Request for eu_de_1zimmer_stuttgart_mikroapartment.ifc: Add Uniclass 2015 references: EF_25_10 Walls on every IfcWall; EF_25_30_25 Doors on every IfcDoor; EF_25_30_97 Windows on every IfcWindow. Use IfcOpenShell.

First a look at what the model holds.

```python
import ifcopenshell

model = ifcopenshell.open("eu_de_1zimmer_stuttgart_mikroapartment.ifc")
print(model.schema)
print("classifications:", [c.Name for c in model.by_type("IfcClassification")])
for ifc_class in ("IfcDoor", "IfcRoof", "IfcStair", "IfcWall", "IfcWindow"):
    print(ifc_class, len(model.by_type(ifc_class)))
```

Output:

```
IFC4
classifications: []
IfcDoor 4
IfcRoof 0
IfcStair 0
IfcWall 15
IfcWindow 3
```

```python
import ifcopenshell
import ifcopenshell.api.classification

model = ifcopenshell.open("eu_de_1zimmer_stuttgart_mikroapartment.ifc")

system = ifcopenshell.api.classification.add_classification(model, classification="Uniclass 2015")

codes = {
    "IfcWall": ("EF_25_10", "Walls"),
    "IfcDoor": ("EF_25_30_25", "Doors"),
    "IfcWindow": ("EF_25_30_97", "Windows"),
}
for ifc_class, (code, name) in codes.items():
    products = model.by_type(ifc_class)
    ifcopenshell.api.classification.add_reference(
        model, products=products, classification=system, identification=code, name=name
    )
    print(code, len(products))

model.write("eu_de_1zimmer_stuttgart_mikroapartment-out.ifc")
```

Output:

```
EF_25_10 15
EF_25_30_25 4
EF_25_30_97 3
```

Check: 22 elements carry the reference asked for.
